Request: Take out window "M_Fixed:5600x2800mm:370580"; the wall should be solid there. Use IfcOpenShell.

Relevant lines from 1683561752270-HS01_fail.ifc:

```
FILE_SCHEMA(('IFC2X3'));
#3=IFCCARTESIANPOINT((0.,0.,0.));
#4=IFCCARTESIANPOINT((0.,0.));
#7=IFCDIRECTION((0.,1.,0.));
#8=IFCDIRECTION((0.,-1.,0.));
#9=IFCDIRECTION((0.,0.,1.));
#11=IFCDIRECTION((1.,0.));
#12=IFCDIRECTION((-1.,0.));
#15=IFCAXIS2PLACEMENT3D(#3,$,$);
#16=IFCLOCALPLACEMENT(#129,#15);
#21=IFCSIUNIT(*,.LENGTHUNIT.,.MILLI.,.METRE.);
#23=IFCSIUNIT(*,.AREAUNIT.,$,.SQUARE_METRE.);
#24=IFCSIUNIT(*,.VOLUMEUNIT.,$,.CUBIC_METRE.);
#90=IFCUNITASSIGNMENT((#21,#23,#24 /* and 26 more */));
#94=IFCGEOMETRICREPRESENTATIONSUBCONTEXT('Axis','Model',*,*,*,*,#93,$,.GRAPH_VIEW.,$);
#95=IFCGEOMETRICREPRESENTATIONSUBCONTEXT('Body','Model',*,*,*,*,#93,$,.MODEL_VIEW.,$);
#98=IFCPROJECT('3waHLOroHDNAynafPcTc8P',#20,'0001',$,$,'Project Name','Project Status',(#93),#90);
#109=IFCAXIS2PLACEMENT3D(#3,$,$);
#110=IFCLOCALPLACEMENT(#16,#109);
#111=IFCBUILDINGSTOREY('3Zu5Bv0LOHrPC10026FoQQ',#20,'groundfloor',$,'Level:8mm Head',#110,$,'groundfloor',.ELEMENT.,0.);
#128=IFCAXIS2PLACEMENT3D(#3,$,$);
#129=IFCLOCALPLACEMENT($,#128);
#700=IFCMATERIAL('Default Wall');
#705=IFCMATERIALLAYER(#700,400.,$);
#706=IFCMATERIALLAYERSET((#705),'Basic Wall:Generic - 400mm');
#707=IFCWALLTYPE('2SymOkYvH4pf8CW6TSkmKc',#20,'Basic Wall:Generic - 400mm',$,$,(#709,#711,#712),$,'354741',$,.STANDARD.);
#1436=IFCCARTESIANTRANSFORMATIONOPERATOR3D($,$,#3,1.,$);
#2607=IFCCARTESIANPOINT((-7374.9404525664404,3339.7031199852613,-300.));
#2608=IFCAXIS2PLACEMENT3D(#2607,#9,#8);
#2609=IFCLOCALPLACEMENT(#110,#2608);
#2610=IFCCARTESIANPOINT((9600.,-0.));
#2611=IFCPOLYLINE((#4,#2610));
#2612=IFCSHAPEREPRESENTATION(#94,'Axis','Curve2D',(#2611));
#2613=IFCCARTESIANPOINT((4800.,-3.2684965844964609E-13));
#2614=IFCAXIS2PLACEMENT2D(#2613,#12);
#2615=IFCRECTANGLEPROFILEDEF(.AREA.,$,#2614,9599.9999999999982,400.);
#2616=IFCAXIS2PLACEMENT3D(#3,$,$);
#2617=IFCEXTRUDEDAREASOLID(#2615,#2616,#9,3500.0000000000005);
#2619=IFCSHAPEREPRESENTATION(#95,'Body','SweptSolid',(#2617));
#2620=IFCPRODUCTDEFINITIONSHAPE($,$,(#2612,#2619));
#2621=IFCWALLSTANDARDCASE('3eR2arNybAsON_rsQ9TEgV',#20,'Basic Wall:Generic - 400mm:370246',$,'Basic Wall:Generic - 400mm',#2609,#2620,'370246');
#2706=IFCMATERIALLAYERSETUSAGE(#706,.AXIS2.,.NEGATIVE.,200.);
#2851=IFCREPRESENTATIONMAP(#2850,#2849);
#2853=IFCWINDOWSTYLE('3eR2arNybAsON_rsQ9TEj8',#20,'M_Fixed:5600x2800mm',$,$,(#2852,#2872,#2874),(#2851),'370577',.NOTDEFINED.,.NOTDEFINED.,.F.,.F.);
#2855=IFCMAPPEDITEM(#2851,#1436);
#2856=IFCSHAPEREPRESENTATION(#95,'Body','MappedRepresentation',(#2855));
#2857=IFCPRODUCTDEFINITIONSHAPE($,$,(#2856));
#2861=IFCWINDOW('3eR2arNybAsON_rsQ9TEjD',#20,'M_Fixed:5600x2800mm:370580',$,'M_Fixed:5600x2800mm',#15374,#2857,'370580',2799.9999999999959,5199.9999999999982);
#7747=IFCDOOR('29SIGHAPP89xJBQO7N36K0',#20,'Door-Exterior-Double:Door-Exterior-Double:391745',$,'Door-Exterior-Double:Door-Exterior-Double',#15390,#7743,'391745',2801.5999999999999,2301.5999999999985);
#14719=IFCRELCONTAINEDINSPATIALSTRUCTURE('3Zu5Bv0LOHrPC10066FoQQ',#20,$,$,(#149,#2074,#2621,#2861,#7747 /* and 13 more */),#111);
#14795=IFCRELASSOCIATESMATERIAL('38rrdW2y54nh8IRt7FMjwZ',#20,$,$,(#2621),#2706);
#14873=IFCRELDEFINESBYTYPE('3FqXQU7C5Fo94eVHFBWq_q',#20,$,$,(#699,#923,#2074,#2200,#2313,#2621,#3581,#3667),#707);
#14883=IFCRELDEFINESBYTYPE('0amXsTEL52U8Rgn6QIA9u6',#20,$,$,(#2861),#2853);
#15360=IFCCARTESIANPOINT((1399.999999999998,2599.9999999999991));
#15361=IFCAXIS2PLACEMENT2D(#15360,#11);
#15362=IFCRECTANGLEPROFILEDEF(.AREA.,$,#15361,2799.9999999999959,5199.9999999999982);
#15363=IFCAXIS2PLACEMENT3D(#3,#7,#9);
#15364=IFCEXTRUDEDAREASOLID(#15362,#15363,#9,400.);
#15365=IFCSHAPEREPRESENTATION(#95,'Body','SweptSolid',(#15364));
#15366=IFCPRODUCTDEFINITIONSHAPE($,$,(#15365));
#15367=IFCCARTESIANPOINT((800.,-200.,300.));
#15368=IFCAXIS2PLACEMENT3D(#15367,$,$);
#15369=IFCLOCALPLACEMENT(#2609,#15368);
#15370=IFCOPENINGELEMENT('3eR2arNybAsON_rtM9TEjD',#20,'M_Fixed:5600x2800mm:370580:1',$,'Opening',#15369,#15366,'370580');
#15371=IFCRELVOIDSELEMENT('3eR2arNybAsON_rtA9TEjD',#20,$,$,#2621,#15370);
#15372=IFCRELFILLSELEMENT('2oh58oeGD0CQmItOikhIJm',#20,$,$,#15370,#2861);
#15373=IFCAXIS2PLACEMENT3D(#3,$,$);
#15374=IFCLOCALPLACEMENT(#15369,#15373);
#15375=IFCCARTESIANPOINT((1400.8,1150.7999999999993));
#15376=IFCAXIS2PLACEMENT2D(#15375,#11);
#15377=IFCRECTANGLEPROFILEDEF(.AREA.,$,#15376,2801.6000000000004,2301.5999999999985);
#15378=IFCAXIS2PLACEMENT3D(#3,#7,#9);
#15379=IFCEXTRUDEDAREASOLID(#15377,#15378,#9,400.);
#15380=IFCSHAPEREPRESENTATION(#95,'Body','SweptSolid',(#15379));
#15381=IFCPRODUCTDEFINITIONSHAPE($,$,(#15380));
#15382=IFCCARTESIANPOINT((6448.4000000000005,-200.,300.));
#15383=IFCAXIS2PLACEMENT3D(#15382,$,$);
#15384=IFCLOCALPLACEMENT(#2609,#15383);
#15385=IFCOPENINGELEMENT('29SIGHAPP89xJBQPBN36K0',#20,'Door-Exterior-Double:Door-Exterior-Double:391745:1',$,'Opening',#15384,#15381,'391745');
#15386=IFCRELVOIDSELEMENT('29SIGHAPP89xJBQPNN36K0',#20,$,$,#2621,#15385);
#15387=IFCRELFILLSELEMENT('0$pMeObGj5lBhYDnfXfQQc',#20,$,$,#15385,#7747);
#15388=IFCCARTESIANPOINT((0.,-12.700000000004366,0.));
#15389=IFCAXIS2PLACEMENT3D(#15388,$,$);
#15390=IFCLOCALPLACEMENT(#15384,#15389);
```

```python
import ifcopenshell
import ifcopenshell.api.feature
import ifcopenshell.api.root
import ifcopenshell.geom
import ifcopenshell.util.shape

model = ifcopenshell.open("1683561752270-HS01_fail.ifc")
settings = ifcopenshell.geom.settings()


def volume(element):
    """Net volume in cubic metres, openings subtracted."""
    shape = ifcopenshell.geom.create_shape(settings, element)
    return ifcopenshell.util.shape.get_volume(shape.geometry)


window = model.by_id(2861)
opening = window.FillsVoids[0].RelatingOpeningElement
wall = opening.VoidsElements[0].RelatingBuildingElement
before = volume(wall)

ifcopenshell.api.root.remove_product(model, product=window)
ifcopenshell.api.feature.remove_feature(model, feature=opening)

after = volume(wall)

print(f"wall volume {before:.3f} -> {after:.3f} m3")

model.write("1683561752270-HS01_fail_rev.ifc")
```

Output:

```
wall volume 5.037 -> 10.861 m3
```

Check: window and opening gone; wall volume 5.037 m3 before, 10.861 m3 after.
